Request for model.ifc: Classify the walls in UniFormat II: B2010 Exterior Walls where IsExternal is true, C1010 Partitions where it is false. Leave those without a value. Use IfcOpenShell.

First a look at what the model holds.

```python
import ifcopenshell
import ifcopenshell.util.element

model = ifcopenshell.open("model.ifc")
print(model.schema)
print("classifications:", [c.Name for c in model.by_type("IfcClassification")])
values = [ifcopenshell.util.element.get_pset(e, "Pset_WallCommon", "IsExternal") for e in model.by_type("IfcWall")]
for value in (True, False, None):
    print("IsExternal", value, values.count(value))
```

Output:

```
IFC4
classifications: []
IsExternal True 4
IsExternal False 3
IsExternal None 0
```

```python
import ifcopenshell
import ifcopenshell.api.classification
import ifcopenshell.util.element

model = ifcopenshell.open("model.ifc")

system = ifcopenshell.api.classification.add_classification(model, classification="UniFormat II")

walls = model.by_type("IfcWall")
external = {e: ifcopenshell.util.element.get_pset(e, "Pset_WallCommon", "IsExternal") for e in walls}
for flag, code, name in ((True, "B2010", "Exterior Walls"), (False, "C1010", "Partitions")):
    products = [e for e in walls if external[e] is flag]
    ifcopenshell.api.classification.add_reference(
        model, products=products, classification=system, identification=code, name=name
    )
    print(code, len(products))

model.write("model_v2.ifc")
```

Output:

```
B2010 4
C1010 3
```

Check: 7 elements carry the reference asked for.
